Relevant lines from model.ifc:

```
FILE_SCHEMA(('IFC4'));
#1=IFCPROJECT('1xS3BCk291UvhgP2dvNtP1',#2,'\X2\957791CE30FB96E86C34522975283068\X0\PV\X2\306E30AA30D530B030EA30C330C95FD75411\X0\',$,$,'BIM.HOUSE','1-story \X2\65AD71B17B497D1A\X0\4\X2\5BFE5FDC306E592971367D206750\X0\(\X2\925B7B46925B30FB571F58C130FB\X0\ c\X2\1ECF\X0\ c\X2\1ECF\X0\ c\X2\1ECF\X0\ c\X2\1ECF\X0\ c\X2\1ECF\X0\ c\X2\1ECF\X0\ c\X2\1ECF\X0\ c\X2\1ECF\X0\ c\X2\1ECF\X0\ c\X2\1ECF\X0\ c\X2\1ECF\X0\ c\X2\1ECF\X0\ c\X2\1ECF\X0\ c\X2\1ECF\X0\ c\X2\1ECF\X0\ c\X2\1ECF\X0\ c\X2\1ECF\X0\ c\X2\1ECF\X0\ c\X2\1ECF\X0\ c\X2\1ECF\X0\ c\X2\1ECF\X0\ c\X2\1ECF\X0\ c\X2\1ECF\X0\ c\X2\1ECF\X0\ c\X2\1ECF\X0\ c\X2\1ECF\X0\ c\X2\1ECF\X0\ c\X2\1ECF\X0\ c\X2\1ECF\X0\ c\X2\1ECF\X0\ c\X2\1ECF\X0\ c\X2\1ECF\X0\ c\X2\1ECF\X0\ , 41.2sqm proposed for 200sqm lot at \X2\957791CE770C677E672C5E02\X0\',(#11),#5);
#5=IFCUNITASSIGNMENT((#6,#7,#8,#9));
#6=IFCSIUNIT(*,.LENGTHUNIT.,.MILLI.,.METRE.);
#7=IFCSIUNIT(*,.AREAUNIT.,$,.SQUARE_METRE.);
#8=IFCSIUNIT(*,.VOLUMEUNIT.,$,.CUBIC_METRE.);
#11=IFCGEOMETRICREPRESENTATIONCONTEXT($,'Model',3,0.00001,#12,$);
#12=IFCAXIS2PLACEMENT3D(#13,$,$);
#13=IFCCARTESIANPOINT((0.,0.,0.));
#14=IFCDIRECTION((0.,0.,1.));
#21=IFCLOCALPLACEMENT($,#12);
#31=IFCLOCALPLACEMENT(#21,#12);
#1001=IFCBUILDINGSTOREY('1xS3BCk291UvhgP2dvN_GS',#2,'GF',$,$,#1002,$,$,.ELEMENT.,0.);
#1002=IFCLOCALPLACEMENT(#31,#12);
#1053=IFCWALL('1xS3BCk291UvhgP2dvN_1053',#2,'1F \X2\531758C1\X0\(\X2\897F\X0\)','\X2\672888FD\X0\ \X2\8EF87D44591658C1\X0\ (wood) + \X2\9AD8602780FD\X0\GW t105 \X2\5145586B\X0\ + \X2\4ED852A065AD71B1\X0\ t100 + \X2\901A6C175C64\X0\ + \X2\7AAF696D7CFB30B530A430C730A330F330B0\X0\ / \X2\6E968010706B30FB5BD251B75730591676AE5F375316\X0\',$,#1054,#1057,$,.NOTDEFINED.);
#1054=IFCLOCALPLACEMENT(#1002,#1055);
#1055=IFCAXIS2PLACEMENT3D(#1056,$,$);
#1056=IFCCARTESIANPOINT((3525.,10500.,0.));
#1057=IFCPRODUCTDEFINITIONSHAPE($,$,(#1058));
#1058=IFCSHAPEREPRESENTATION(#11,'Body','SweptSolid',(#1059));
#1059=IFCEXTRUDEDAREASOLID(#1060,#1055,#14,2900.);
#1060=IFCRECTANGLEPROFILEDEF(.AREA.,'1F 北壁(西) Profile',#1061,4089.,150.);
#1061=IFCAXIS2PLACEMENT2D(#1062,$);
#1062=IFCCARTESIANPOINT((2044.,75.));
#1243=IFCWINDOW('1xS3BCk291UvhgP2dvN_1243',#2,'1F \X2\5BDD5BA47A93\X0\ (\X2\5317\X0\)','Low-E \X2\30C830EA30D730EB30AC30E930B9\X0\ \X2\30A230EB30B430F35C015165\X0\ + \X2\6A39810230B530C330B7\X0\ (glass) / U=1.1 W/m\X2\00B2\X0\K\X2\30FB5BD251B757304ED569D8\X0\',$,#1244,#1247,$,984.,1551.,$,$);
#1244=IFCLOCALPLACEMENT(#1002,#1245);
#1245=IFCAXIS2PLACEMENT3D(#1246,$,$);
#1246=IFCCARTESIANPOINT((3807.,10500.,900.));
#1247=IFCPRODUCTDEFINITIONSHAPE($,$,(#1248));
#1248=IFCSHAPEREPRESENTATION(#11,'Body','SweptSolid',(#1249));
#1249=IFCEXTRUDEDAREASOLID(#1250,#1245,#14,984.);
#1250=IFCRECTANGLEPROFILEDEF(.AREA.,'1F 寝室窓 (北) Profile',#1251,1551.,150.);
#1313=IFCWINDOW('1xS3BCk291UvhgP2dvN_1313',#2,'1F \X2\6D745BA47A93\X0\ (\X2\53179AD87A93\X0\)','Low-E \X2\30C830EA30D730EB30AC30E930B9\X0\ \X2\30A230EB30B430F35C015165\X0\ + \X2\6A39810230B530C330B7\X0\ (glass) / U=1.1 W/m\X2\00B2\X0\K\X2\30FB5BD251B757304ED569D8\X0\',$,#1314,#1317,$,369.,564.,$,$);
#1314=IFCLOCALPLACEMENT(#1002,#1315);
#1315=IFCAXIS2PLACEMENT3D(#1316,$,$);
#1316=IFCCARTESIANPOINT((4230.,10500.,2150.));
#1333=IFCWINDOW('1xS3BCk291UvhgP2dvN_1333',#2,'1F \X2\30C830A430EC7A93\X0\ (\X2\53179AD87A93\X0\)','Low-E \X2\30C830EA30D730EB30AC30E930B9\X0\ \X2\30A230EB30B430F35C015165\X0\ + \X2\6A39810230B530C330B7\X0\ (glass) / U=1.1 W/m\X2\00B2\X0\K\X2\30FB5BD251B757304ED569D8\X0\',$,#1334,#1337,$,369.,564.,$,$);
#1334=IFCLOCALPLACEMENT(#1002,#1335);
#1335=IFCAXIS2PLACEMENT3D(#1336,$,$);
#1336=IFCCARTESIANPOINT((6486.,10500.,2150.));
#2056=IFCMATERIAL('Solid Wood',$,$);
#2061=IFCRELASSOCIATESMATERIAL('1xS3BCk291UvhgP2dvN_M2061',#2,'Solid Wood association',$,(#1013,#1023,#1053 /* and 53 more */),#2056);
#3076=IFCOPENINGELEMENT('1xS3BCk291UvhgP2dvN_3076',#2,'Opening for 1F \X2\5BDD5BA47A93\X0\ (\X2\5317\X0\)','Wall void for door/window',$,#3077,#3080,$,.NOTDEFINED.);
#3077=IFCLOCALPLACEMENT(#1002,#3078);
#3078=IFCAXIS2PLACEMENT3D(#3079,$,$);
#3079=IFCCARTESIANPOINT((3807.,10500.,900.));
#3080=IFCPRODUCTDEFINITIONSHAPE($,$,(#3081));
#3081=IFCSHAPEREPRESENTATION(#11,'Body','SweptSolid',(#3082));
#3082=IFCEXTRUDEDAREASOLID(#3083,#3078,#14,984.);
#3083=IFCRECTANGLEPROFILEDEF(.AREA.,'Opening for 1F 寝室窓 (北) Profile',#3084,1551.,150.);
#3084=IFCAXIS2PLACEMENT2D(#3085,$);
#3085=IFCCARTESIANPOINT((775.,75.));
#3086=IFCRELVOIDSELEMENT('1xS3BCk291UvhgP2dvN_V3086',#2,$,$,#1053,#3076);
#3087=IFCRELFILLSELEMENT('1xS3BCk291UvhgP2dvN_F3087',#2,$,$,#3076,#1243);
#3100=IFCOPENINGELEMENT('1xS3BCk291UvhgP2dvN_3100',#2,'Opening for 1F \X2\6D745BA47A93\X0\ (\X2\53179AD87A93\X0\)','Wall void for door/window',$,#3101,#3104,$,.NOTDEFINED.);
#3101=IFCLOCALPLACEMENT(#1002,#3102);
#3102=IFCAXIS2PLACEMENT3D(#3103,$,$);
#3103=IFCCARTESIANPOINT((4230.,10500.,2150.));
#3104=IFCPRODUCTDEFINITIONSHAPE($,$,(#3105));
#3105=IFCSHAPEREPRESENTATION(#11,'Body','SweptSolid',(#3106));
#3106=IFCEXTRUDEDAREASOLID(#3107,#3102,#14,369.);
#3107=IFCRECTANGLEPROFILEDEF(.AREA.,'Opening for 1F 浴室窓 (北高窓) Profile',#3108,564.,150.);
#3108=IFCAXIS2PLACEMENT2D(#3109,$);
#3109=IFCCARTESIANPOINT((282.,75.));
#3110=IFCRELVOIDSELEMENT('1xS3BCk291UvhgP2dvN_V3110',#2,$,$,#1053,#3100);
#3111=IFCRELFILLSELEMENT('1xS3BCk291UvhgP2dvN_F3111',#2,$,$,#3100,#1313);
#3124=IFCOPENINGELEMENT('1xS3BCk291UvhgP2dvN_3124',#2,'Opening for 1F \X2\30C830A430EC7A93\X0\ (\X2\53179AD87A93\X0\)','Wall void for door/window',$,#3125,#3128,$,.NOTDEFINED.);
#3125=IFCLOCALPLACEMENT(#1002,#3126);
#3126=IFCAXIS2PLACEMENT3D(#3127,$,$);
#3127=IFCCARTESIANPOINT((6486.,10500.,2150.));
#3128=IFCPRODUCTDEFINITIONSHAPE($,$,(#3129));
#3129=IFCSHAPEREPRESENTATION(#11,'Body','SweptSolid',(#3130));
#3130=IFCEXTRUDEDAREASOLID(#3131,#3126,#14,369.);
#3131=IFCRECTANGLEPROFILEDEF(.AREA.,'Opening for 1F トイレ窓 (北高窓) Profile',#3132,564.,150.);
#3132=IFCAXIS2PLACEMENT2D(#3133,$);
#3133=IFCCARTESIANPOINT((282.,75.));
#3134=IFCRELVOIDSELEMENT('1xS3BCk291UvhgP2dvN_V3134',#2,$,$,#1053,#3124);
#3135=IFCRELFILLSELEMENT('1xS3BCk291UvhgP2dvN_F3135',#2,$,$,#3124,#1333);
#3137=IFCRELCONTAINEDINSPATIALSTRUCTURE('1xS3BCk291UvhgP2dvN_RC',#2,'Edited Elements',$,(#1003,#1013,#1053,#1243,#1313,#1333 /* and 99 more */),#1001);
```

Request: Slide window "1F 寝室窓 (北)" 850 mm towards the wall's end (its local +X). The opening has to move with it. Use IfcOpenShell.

```python
import ifcopenshell
import ifcopenshell.api.geometry
import ifcopenshell.util.placement

model = ifcopenshell.open("model.ifc")

window = model.by_guid("1xS3BCk291UvhgP2dvN_1243")
opening = window.FillsVoids[0].RelatingOpeningElement
wall = opening.VoidsElements[0].RelatingBuildingElement

wall_matrix = ifcopenshell.util.placement.get_local_placement(wall.ObjectPlacement)
shift = wall_matrix[:3, 0] * 850.0
before = ifcopenshell.util.placement.get_local_placement(window.ObjectPlacement)[:3, 3].copy()

# The window is not placed relative to its opening, so move both.
for product in (opening, window):
    matrix = ifcopenshell.util.placement.get_local_placement(product.ObjectPlacement)
    matrix[:3, 3] += shift
    ifcopenshell.api.geometry.edit_object_placement(model, product=product, matrix=matrix, is_si=False)

after = ifcopenshell.util.placement.get_local_placement(window.ObjectPlacement)[:3, 3]
print("window moved by", (after - before).round(3) + 0.0)

model.write("model_edited.ifc")
```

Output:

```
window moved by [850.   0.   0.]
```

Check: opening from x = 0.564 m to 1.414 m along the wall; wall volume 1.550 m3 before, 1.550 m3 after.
